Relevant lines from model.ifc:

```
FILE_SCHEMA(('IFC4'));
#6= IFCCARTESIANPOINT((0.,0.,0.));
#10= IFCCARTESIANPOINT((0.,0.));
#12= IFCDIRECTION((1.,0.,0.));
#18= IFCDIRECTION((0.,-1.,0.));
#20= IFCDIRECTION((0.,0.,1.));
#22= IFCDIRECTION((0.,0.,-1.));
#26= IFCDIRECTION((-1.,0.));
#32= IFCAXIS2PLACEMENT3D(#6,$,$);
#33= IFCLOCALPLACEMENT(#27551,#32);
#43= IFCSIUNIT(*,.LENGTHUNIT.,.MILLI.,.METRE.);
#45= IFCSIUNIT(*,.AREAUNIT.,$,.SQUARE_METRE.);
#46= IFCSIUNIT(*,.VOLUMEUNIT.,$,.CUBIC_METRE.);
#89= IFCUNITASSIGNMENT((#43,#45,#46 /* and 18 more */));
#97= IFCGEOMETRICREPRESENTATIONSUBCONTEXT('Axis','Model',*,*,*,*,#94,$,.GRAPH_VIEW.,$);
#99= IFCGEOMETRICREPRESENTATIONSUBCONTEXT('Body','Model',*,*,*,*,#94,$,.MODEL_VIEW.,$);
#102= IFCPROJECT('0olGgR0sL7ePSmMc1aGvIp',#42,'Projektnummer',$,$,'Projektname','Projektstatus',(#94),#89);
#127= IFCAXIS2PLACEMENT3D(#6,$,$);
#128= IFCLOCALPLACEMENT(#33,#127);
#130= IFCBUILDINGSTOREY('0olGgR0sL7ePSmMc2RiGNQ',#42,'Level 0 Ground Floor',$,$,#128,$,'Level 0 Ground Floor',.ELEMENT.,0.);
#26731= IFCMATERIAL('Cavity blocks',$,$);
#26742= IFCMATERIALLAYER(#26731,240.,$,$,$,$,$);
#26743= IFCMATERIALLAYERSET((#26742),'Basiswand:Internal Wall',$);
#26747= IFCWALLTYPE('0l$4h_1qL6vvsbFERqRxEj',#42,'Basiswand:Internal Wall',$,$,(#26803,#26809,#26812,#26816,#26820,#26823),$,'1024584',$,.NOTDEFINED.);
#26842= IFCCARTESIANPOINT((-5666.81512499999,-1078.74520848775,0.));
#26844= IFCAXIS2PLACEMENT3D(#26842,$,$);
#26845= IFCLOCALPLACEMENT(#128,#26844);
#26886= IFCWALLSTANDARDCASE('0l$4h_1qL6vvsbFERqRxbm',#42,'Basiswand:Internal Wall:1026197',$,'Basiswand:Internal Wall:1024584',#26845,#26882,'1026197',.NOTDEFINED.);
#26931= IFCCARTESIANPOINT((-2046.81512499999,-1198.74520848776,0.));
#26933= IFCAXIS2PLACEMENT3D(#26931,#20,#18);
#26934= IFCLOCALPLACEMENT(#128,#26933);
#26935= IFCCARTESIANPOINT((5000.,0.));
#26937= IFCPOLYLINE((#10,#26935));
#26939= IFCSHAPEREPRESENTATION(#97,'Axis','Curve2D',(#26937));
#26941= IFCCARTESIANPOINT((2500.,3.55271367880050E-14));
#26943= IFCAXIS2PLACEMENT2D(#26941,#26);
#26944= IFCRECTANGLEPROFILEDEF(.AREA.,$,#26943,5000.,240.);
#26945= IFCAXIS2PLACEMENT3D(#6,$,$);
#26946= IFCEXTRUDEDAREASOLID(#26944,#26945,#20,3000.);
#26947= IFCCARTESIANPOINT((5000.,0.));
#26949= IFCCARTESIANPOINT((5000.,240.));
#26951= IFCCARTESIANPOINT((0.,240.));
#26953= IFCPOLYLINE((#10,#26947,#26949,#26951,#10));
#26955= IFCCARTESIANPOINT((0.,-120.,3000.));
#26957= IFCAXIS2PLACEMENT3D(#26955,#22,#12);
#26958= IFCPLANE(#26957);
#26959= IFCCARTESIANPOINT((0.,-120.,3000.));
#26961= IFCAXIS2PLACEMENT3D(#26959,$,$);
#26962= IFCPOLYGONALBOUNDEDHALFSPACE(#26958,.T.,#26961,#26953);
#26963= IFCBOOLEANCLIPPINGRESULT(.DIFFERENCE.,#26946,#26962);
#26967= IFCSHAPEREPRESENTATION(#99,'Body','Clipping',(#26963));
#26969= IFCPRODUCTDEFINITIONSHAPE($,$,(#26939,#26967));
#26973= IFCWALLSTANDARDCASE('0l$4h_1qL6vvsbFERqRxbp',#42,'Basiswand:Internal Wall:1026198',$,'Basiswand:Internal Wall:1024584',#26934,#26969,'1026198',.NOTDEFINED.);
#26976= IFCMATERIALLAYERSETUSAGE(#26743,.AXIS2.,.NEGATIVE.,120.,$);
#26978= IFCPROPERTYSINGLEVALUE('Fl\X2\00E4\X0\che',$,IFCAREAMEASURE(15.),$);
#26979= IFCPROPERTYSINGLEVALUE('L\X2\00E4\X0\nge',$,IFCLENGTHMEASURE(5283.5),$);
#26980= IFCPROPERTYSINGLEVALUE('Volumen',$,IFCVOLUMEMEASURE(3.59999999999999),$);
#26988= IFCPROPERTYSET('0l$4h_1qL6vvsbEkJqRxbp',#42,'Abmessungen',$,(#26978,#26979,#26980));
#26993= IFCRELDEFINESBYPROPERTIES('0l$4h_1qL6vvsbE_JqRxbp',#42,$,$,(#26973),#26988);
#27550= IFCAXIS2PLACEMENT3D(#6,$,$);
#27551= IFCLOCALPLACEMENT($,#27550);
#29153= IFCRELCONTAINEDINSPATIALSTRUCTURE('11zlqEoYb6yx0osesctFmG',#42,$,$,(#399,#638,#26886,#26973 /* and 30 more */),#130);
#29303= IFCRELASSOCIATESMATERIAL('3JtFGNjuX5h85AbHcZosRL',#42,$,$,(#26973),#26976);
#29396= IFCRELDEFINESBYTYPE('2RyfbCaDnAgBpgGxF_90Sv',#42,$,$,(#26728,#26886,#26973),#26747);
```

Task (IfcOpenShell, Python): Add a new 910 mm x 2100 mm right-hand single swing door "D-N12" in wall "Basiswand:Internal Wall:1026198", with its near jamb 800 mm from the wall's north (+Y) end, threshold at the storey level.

```python
import numpy as np
import ifcopenshell
import ifcopenshell.api.feature
import ifcopenshell.api.geometry
import ifcopenshell.api.pset
import ifcopenshell.api.root
import ifcopenshell.api.spatial
import ifcopenshell.geom
import ifcopenshell.util.element
import ifcopenshell.util.placement
import ifcopenshell.util.representation
import ifcopenshell.util.shape
import ifcopenshell.util.unit

model = ifcopenshell.open("model.ifc")
unit_scale = ifcopenshell.util.unit.calculate_unit_scale(model)
area_scale = ifcopenshell.util.unit.calculate_unit_scale(model, "AREAUNIT")
volume_scale = ifcopenshell.util.unit.calculate_unit_scale(model, "VOLUMEUNIT")
settings = ifcopenshell.geom.settings()


def volume(element):
    """Net volume in cubic metres, openings subtracted."""
    shape = ifcopenshell.geom.create_shape(settings, element)
    return ifcopenshell.util.shape.get_volume(shape.geometry)


wall = model.by_guid("0l$4h_1qL6vvsbFERqRxbp")
storey = ifcopenshell.util.element.get_container(wall, ifc_class="IfcBuildingStorey")
context = ifcopenshell.util.representation.get_context(model, "Model", "Body", "MODEL_VIEW")
before = volume(wall)

width, height, from_end, sill = 0.91, 2.1, 0.8, 0.0  # metres

# The wall runs along its own X axis, and the end named is its -X end.
wall_shape = ifcopenshell.geom.create_shape(settings, wall)
x, y, z = ifcopenshell.util.shape.get_vertices(wall_shape.geometry).T
start = x.min() + from_end
face, thickness = float(y.min()), float(y.max() - y.min())
wall_matrix = ifcopenshell.util.placement.get_local_placement(wall.ObjectPlacement)
level = ifcopenshell.util.placement.get_local_placement(storey.ObjectPlacement)[2, 3]


def in_wall(x, y):
    """Placement at x, y metres in the wall's axes, at sill height."""
    matrix = wall_matrix.copy()
    matrix[:, 3] = wall_matrix @ np.array([x / unit_scale, y / unit_scale, 0.0, 1.0])
    matrix[2, 3] = level + sill / unit_scale
    return matrix


# Opening: a box that overshoots both wall faces by 50 mm.
opening = ifcopenshell.api.root.create_entity(model, ifc_class="IfcOpeningElement", predefined_type="OPENING")
box = ifcopenshell.api.geometry.add_wall_representation(
    model, context=context, length=width, height=height, thickness=thickness + 0.1
)
ifcopenshell.api.geometry.assign_representation(model, product=opening, representation=box)
ifcopenshell.api.geometry.edit_object_placement(model, product=opening, matrix=in_wall(start, face - 0.05), is_si=False)
ifcopenshell.api.feature.add_feature(model, feature=opening, element=wall)

door = ifcopenshell.api.root.create_entity(model, ifc_class="IfcDoor", name="D-N12", predefined_type="DOOR")
door.OverallWidth, door.OverallHeight = width / unit_scale, height / unit_scale
door.OperationType = "SINGLE_SWING_RIGHT"
body = ifcopenshell.api.geometry.add_door_representation(
    model,
    context=context,
    overall_width=door.OverallWidth,
    overall_height=door.OverallHeight,
    operation_type="SINGLE_SWING_RIGHT",
    lining_properties={"LiningDepth": thickness / unit_scale, "ThresholdDepth": thickness / unit_scale},
)
ifcopenshell.api.geometry.assign_representation(model, product=door, representation=body)
ifcopenshell.api.spatial.assign_container(model, products=[door], relating_structure=storey)
ifcopenshell.api.feature.add_filling(model, opening=opening, element=door)

# The lining spans the wall, so the door starts at the wall face.
ifcopenshell.api.geometry.edit_object_placement(model, product=door, matrix=in_wall(start, face), is_si=False)

after = volume(wall)

# Update the wall's stored quantities.
pset = model.by_id(ifcopenshell.util.element.get_pset(wall, "Abmessungen", should_inherit=False)["id"])
ifcopenshell.api.pset.edit_pset(model, pset=pset, properties={
    "Fläche": model.create_entity("IfcAreaMeasure", after / thickness / area_scale),
    "Volumen": model.create_entity("IfcVolumeMeasure", after / volume_scale),
})

print(f"wall volume {before:.3f} -> {after:.3f} m3")

model.write("model_updated.ifc")
```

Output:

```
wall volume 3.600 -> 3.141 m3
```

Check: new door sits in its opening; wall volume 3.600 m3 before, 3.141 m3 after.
